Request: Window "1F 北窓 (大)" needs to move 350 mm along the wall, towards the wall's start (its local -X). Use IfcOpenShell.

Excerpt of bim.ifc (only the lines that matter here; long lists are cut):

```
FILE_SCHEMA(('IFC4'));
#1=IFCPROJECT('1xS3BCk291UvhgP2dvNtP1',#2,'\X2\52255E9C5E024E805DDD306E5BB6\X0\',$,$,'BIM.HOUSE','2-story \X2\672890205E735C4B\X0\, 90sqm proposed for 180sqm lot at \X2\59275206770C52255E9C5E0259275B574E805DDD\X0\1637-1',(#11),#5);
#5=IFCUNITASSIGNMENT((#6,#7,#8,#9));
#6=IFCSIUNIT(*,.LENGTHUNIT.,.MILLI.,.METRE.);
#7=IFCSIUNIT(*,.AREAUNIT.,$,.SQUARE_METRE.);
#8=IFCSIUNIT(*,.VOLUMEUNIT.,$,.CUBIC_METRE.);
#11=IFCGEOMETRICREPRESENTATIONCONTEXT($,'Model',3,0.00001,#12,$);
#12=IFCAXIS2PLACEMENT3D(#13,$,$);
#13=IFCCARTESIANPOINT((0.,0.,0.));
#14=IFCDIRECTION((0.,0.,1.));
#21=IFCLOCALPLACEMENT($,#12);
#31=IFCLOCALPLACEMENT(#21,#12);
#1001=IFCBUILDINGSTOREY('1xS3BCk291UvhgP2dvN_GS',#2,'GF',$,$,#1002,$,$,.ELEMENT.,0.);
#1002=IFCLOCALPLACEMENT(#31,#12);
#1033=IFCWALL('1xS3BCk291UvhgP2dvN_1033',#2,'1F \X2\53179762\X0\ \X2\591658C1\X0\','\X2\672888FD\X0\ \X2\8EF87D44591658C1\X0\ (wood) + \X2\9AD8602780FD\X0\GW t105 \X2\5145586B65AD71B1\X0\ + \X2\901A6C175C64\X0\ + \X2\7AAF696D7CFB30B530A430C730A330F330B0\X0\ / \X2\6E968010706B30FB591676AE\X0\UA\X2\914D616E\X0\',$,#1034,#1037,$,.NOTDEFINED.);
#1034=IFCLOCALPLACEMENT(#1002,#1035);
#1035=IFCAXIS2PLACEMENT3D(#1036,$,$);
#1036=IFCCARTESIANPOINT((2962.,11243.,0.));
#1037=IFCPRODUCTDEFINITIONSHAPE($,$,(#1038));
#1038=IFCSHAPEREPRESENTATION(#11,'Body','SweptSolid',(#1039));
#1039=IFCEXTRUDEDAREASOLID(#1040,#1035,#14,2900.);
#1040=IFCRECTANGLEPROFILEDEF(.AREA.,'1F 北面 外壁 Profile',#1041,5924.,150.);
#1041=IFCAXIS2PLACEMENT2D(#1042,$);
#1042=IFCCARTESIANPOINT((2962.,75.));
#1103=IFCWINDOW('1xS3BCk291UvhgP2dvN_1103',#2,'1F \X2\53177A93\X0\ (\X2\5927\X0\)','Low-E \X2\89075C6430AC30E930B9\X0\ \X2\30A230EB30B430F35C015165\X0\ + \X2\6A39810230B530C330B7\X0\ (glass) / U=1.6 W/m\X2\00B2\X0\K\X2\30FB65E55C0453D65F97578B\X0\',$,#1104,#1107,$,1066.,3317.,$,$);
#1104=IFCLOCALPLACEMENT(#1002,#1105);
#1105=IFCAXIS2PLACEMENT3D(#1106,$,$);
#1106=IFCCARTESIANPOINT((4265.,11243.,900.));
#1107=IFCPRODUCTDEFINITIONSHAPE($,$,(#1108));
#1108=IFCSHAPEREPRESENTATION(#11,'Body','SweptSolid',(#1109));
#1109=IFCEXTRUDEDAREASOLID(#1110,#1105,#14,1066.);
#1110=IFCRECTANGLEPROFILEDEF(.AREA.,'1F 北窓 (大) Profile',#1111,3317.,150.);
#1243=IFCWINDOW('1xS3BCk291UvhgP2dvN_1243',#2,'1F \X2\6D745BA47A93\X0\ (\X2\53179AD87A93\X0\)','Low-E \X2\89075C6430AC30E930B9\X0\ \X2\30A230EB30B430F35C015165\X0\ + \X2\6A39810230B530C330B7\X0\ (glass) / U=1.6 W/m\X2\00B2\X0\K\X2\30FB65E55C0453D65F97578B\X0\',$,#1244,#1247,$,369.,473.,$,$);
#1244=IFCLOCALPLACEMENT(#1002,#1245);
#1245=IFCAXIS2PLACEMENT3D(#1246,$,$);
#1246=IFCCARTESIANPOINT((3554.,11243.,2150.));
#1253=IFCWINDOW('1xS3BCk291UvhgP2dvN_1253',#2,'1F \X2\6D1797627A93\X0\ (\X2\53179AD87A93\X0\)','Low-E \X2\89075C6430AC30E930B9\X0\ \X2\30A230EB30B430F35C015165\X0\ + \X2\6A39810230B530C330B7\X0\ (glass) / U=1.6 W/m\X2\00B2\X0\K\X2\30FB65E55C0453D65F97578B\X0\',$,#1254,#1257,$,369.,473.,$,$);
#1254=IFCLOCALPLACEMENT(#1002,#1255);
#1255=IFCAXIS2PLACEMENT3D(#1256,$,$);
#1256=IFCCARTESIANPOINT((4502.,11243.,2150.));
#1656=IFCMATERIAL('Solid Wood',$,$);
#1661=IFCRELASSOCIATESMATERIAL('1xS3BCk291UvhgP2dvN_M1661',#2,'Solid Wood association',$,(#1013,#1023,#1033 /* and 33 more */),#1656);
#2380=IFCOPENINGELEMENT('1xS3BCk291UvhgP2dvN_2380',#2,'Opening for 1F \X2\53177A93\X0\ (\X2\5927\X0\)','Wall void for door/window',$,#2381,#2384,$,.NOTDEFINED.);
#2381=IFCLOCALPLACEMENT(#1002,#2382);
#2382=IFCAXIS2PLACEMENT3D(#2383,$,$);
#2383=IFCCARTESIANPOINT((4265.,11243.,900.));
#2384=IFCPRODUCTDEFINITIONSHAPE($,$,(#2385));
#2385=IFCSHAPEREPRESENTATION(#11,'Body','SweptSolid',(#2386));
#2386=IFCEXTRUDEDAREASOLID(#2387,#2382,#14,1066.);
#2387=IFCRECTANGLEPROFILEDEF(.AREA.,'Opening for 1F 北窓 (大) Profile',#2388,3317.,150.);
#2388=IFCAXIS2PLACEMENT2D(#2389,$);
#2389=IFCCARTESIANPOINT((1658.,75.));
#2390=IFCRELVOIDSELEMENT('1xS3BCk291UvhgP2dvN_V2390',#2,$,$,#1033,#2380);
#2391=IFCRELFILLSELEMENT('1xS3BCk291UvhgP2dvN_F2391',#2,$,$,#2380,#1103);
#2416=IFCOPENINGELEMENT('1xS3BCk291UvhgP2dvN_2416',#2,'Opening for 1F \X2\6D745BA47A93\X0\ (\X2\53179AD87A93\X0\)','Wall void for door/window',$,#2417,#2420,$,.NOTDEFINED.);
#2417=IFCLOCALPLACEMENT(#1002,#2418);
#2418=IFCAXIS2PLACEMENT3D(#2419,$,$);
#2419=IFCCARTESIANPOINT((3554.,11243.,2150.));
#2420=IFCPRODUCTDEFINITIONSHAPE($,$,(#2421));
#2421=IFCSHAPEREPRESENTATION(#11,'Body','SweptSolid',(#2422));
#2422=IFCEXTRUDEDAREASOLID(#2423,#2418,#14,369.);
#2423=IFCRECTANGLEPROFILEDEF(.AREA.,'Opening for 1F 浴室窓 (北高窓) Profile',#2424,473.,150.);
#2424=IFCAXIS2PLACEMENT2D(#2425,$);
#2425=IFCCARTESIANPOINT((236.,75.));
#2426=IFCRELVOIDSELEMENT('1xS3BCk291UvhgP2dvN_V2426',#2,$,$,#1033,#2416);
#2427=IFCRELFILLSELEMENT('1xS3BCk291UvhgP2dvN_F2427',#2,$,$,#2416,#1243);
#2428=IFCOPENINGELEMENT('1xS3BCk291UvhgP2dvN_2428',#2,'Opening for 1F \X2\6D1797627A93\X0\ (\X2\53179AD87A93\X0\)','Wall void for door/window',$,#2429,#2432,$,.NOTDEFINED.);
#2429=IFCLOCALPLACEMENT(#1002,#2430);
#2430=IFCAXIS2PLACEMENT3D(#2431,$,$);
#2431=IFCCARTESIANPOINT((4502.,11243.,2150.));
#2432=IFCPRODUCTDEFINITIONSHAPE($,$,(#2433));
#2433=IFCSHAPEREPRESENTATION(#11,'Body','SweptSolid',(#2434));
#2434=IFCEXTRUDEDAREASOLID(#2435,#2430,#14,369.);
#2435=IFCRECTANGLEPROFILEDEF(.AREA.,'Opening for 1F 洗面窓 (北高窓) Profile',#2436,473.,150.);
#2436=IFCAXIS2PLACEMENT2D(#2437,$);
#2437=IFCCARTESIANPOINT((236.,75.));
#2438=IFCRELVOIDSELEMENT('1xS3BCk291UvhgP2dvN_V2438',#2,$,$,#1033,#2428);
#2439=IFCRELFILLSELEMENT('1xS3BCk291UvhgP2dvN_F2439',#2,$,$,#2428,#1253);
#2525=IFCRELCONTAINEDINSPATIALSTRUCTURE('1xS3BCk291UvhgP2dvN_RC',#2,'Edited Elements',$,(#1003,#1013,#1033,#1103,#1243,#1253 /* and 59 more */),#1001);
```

```python
import ifcopenshell
import ifcopenshell.api.geometry
import ifcopenshell.util.placement
import ifcopenshell.util.unit

model = ifcopenshell.open("bim.ifc")
unit_scale = ifcopenshell.util.unit.calculate_unit_scale(model)

window = model.by_guid("1xS3BCk291UvhgP2dvN_1103")
opening = window.FillsVoids[0].RelatingOpeningElement
wall = opening.VoidsElements[0].RelatingBuildingElement

wall_matrix = ifcopenshell.util.placement.get_local_placement(wall.ObjectPlacement)
shift = wall_matrix[:3, 0] * -0.35 / unit_scale
before = ifcopenshell.util.placement.get_local_placement(window.ObjectPlacement)[:3, 3].copy()

# The window is not placed relative to its opening, so move both.
for product in (opening, window):
    matrix = ifcopenshell.util.placement.get_local_placement(product.ObjectPlacement)
    matrix[:3, 3] += shift
    ifcopenshell.api.geometry.edit_object_placement(model, product=product, matrix=matrix, is_si=False)

after = ifcopenshell.util.placement.get_local_placement(window.ObjectPlacement)[:3, 3]
print("window moved by", (after - before).round(3) + 0.0)

model.write("bim-out.ifc")
```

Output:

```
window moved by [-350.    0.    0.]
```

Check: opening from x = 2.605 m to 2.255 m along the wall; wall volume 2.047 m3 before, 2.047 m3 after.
